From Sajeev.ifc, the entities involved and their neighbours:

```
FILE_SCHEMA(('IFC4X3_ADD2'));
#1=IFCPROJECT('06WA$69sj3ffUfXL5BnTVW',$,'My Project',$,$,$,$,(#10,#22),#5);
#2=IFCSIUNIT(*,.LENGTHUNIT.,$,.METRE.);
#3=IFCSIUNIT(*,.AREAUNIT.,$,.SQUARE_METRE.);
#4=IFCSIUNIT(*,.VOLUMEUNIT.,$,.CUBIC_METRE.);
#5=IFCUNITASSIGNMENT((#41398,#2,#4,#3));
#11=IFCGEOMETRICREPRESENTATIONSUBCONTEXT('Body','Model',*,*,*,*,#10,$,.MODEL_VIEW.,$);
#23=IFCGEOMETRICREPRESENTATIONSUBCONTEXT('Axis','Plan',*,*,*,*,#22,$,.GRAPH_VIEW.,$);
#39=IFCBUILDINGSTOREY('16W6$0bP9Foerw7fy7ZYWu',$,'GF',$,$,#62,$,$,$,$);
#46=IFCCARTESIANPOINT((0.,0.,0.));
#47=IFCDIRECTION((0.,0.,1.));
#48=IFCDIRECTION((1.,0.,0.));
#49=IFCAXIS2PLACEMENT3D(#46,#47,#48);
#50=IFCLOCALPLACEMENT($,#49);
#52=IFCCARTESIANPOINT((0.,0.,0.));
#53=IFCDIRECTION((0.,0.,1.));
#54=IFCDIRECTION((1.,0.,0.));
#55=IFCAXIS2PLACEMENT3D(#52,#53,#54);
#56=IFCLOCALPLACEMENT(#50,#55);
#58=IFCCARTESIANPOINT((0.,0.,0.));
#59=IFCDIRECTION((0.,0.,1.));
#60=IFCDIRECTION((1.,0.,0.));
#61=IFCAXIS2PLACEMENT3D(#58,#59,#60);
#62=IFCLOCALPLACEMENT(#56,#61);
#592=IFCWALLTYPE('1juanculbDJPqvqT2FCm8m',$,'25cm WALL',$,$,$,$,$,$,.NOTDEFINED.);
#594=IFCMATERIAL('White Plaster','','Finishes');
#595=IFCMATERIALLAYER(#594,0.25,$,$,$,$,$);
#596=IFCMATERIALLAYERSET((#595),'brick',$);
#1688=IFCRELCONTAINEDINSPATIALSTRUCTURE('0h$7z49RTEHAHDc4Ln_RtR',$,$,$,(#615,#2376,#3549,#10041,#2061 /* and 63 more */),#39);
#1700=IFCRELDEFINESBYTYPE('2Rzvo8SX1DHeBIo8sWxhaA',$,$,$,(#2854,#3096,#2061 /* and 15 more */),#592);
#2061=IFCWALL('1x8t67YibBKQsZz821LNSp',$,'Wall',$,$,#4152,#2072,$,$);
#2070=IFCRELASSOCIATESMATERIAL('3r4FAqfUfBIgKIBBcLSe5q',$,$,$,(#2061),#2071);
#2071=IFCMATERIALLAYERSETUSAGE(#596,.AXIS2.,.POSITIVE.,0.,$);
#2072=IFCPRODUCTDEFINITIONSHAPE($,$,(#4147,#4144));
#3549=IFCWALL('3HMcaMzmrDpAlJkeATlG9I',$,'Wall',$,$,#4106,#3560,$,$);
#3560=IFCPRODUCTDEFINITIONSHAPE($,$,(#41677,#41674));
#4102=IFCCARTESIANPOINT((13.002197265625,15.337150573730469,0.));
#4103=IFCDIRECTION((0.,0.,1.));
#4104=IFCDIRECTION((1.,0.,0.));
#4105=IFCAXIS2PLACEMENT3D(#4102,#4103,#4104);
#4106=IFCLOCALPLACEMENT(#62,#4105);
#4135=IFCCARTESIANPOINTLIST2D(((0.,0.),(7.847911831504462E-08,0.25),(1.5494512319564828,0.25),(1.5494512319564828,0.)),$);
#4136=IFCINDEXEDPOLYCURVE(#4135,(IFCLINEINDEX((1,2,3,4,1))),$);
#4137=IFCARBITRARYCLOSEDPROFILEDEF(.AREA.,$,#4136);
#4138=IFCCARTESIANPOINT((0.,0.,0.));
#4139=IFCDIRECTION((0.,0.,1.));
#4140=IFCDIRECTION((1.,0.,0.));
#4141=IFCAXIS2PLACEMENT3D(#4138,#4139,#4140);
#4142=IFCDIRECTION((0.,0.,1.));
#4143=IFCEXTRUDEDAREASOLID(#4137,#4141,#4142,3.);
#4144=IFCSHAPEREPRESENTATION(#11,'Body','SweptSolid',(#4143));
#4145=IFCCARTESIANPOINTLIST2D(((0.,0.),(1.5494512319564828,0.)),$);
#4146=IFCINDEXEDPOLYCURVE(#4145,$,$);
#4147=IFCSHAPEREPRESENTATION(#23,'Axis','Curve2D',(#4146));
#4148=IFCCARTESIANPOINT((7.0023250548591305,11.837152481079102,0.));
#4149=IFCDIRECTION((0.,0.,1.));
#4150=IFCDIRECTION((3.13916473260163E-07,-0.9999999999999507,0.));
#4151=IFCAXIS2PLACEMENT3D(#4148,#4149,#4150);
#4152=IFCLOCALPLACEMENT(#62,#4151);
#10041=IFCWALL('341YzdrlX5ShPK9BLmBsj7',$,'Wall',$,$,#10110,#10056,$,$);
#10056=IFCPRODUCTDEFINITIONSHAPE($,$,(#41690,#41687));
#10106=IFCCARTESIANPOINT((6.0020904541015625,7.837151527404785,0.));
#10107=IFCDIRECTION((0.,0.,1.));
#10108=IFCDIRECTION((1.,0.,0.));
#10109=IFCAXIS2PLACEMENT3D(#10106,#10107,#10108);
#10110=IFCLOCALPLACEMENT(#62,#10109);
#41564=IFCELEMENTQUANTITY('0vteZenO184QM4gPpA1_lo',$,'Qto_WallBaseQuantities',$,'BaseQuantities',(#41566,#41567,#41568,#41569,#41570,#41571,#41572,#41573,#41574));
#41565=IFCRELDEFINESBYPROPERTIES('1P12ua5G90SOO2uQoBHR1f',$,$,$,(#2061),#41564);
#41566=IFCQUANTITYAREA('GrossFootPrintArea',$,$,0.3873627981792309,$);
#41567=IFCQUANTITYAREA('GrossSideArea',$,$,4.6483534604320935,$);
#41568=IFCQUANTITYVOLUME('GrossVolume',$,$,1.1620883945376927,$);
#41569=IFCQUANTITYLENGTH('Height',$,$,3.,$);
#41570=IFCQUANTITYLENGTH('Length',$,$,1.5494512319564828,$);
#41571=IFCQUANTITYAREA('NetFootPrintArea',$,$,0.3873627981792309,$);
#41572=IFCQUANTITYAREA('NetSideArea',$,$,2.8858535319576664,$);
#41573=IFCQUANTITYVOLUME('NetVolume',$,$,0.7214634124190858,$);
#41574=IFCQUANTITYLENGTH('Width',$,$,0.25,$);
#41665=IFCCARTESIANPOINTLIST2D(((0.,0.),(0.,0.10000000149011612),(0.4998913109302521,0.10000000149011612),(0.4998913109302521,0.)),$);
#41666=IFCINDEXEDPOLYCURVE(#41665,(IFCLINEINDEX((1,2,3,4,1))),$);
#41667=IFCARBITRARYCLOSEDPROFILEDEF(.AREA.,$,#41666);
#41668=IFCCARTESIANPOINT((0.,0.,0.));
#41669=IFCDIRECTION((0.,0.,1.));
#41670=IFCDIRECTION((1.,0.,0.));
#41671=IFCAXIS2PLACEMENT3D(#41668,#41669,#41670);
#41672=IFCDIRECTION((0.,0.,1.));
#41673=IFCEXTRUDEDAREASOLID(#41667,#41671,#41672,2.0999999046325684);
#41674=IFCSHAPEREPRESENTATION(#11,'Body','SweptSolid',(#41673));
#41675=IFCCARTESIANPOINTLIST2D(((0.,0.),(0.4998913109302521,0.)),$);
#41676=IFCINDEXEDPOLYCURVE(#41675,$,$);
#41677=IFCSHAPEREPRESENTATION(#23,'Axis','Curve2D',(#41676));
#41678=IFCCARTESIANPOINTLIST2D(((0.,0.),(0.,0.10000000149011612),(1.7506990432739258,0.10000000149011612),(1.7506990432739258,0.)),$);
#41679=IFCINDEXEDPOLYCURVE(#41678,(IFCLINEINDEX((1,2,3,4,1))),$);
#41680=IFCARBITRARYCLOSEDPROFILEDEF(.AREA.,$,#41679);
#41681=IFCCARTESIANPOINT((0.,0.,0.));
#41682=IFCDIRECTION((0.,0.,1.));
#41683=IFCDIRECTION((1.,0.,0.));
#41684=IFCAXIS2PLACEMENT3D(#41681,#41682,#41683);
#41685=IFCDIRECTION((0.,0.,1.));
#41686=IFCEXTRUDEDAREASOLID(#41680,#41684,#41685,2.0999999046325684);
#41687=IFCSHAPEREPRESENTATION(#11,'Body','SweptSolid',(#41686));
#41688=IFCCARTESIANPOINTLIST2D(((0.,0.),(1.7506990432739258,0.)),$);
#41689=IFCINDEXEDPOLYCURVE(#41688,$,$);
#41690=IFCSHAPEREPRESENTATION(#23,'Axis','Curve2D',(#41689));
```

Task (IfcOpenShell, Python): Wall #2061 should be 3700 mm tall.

```python
import ifcopenshell
import ifcopenshell.api.pset
import ifcopenshell.geom
import ifcopenshell.util.element
import ifcopenshell.util.representation
import ifcopenshell.util.shape
import ifcopenshell.util.unit

model = ifcopenshell.open("Sajeev.ifc")
unit_scale = ifcopenshell.util.unit.calculate_unit_scale(model)
area_scale = ifcopenshell.util.unit.calculate_unit_scale(model, "AREAUNIT")
volume_scale = ifcopenshell.util.unit.calculate_unit_scale(model, "VOLUMEUNIT")
settings = ifcopenshell.geom.settings()


def volume(element):
    """Net volume in cubic metres, openings subtracted."""
    shape = ifcopenshell.geom.create_shape(settings, element)
    return ifcopenshell.util.shape.get_volume(shape.geometry)


wall = model.by_id(2061)
before = volume(wall)

body = ifcopenshell.util.representation.get_representation(wall, "Model", "Body")
solid = body.Items[0]
old_height = solid.Depth
solid.Depth = 3.7
after = volume(wall)
thickness = 0.25  # wall thickness in metres

# Update the stored height, areas and volumes.
qto = model.by_id(ifcopenshell.util.element.get_pset(wall, "Qto_WallBaseQuantities", should_inherit=False)["id"])
ifcopenshell.api.pset.edit_qto(model, qto=qto, properties={
    "GrossSideArea": ifcopenshell.util.element.get_pset(wall, "Qto_WallBaseQuantities", "GrossSideArea") * solid.Depth / old_height,
    "GrossVolume": ifcopenshell.util.element.get_pset(wall, "Qto_WallBaseQuantities", "GrossVolume") * solid.Depth / old_height,
    "Height": solid.Depth,
    "NetSideArea": after / thickness / area_scale,
    "NetVolume": after / volume_scale,
})

print(f"height {old_height:g} -> {solid.Depth:g}, volume {before:.3f} -> {after:.3f} m3")

model.write("Sajeev_edited.ifc")
```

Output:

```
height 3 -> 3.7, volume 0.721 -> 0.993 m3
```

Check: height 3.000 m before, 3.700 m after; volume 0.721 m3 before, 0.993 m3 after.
